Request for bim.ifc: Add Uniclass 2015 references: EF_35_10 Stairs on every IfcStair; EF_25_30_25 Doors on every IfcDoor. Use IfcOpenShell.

First a look at what the model holds.

```python
import ifcopenshell

model = ifcopenshell.open("bim.ifc")
print(model.schema)
print("classifications:", [c.Name for c in model.by_type("IfcClassification")])
for ifc_class in ("IfcDoor", "IfcRoof", "IfcStair", "IfcWall", "IfcWindow"):
    print(ifc_class, len(model.by_type(ifc_class)))
```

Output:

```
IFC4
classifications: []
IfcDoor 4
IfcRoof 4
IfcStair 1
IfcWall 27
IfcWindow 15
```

```python
import ifcopenshell
import ifcopenshell.api.classification

model = ifcopenshell.open("bim.ifc")

system = ifcopenshell.api.classification.add_classification(model, classification="Uniclass 2015")

codes = {
    "IfcStair": ("EF_35_10", "Stairs"),
    "IfcDoor": ("EF_25_30_25", "Doors"),
}
for ifc_class, (code, name) in codes.items():
    products = model.by_type(ifc_class)
    ifcopenshell.api.classification.add_reference(
        model, products=products, classification=system, identification=code, name=name
    )
    print(code, len(products))

model.write("bim_updated.ifc")
```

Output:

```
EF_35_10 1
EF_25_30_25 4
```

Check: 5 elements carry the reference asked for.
